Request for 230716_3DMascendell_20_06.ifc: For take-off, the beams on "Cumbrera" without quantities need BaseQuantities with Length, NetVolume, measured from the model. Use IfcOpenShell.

First a look at what the model holds.

```python
import ifcopenshell
import ifcopenshell.util.element
import ifcopenshell.util.unit

model = ifcopenshell.open("230716_3DMascendell_20_06.ifc")
print(model.schema)
for unit_type in ("LENGTHUNIT", "AREAUNIT", "VOLUMEUNIT"):
    print(unit_type, ifcopenshell.util.unit.calculate_unit_scale(model, unit_type))
storey = next(s for s in model.by_type("IfcBuildingStorey") if s.Name == "Cumbrera")
beams = [e for e in ifcopenshell.util.element.get_decomposition(storey) if e.is_a("IfcBeam")]
for e in sorted(beams, key=lambda e: e.id()):
    print(e.id(), e.is_a(), e.Name, list(ifcopenshell.util.element.get_psets(e, qtos_only=True)), sep=" | ")
```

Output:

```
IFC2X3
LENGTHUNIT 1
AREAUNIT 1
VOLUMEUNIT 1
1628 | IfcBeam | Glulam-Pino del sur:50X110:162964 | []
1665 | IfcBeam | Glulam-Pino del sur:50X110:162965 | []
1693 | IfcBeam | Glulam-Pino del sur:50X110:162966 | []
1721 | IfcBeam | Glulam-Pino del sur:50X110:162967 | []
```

```python
import ifcopenshell
import ifcopenshell.api.pset
import ifcopenshell.geom
import ifcopenshell.util.element
import ifcopenshell.util.shape
import ifcopenshell.util.unit

model = ifcopenshell.open("230716_3DMascendell_20_06.ifc")
unit_scale = ifcopenshell.util.unit.calculate_unit_scale(model)
volume_scale = ifcopenshell.util.unit.calculate_unit_scale(model, "VOLUMEUNIT")
settings = ifcopenshell.geom.settings()

storey = next(s for s in model.by_type("IfcBuildingStorey") if s.Name == "Cumbrera")
beams = [e for e in ifcopenshell.util.element.get_decomposition(storey) if e.is_a("IfcBeam")]

for e in sorted(beams, key=lambda e: e.id()):
    if ifcopenshell.util.element.get_psets(e, qtos_only=True, should_inherit=False):
        continue
    # Geometry comes back in metres, in the element's own axes.
    shape = ifcopenshell.geom.create_shape(settings, e)
    values = {
        "Length": ifcopenshell.util.shape.get_max_xyz(shape.geometry) / unit_scale,
        "NetVolume": ifcopenshell.util.shape.get_volume(shape.geometry) / volume_scale,
    }
    qto = ifcopenshell.api.pset.add_qto(model, product=e, name="BaseQuantities")
    ifcopenshell.api.pset.edit_qto(model, qto=qto, properties=values)
    print(e.id(), {k: round(v, 3) for k, v in values.items()})

model.write("230716_3DMascendell_20_06_v2.ifc")
```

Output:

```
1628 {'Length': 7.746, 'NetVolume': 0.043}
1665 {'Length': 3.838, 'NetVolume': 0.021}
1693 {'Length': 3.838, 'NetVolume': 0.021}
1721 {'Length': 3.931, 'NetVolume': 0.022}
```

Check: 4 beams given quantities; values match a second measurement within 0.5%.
